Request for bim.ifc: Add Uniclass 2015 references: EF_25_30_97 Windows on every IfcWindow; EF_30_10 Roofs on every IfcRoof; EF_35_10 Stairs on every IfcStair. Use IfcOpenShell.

First a look at what the model holds.

```python
import ifcopenshell

model = ifcopenshell.open("bim.ifc")
print(model.schema)
print("classifications:", [c.Name for c in model.by_type("IfcClassification")])
for ifc_class in ("IfcDoor", "IfcRoof", "IfcStair", "IfcWall", "IfcWindow"):
    print(ifc_class, len(model.by_type(ifc_class)))
```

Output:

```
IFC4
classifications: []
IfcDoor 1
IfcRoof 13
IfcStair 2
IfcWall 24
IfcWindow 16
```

```python
import ifcopenshell
import ifcopenshell.api.classification

model = ifcopenshell.open("bim.ifc")

system = ifcopenshell.api.classification.add_classification(model, classification="Uniclass 2015")

codes = {
    "IfcWindow": ("EF_25_30_97", "Windows"),
    "IfcRoof": ("EF_30_10", "Roofs"),
    "IfcStair": ("EF_35_10", "Stairs"),
}
for ifc_class, (code, name) in codes.items():
    products = model.by_type(ifc_class)
    ifcopenshell.api.classification.add_reference(
        model, products=products, classification=system, identification=code, name=name
    )
    print(code, len(products))

model.write("bim-out.ifc")
```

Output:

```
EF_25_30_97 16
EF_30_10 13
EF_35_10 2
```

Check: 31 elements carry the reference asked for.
